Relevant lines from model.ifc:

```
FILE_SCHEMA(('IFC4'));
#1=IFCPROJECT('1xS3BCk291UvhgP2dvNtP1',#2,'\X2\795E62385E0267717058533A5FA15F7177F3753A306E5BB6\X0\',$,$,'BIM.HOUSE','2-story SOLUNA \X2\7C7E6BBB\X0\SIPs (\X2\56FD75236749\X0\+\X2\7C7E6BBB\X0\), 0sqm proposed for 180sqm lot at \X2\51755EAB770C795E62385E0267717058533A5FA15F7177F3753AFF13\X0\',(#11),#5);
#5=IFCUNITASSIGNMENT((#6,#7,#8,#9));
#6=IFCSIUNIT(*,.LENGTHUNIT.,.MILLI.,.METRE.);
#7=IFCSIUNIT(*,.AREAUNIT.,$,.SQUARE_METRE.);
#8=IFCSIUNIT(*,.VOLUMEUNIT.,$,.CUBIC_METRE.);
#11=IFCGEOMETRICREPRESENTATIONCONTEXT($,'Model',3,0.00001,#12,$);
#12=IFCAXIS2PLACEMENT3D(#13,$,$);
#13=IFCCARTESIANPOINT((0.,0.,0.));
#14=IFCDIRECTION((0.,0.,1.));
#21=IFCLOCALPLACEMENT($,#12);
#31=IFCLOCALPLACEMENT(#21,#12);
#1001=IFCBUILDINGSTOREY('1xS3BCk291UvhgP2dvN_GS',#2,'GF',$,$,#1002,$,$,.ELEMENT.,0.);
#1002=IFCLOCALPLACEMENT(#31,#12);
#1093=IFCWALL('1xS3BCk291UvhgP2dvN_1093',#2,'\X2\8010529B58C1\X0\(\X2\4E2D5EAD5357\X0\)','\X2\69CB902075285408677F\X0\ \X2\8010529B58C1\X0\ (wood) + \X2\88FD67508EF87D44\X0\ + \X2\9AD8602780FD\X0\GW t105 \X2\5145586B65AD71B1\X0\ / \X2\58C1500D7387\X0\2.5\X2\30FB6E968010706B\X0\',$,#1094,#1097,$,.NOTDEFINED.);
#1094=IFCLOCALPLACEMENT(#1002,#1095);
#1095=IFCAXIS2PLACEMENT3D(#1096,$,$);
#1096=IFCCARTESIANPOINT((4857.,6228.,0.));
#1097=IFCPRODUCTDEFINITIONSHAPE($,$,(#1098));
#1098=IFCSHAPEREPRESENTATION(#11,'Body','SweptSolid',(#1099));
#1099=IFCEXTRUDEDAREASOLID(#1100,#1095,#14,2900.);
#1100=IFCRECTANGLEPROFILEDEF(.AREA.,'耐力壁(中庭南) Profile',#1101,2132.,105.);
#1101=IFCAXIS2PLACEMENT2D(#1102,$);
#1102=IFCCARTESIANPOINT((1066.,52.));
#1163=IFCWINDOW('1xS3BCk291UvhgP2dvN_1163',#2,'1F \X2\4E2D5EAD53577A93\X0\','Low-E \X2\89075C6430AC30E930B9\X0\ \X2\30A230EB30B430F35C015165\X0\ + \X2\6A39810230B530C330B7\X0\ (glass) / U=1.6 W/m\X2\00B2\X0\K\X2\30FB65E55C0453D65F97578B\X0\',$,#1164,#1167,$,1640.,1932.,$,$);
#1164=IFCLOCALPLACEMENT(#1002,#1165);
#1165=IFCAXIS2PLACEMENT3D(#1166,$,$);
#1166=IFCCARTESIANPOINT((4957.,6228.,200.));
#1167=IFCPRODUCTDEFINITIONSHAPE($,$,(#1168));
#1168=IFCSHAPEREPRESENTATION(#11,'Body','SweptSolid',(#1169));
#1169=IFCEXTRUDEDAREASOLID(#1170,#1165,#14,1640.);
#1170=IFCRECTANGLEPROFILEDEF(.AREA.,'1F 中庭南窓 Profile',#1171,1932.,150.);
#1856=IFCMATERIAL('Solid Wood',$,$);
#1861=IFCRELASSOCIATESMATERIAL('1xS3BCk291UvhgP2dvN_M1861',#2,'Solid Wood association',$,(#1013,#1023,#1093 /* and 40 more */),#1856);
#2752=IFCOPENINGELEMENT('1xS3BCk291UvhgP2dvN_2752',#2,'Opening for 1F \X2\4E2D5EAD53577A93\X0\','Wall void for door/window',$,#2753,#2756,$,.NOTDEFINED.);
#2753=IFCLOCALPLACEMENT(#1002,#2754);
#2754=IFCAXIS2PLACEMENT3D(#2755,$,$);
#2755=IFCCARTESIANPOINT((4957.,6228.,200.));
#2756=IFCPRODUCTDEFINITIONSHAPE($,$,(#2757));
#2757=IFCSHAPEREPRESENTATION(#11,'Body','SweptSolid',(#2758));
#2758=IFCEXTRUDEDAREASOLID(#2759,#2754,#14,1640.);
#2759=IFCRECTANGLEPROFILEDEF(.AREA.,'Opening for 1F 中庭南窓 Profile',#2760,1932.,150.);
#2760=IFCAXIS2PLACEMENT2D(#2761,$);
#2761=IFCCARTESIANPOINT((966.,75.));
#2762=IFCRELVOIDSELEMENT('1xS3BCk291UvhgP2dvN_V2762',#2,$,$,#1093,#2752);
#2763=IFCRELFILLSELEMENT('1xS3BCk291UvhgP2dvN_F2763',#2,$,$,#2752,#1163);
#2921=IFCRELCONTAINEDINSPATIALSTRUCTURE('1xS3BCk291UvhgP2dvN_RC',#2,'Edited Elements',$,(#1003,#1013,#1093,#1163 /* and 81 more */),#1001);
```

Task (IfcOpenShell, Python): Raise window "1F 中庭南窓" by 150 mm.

```python
import numpy as np
import ifcopenshell
import ifcopenshell.api.geometry
import ifcopenshell.util.placement
import ifcopenshell.util.unit

model = ifcopenshell.open("model.ifc")
unit_scale = ifcopenshell.util.unit.calculate_unit_scale(model)

window = model.by_guid("1xS3BCk291UvhgP2dvN_1163")
opening = window.FillsVoids[0].RelatingOpeningElement
dz = 0.15 / unit_scale

shift = np.array([0.0, 0.0, dz])
# The window is not placed relative to its opening, so move both.
for product in (opening, window):
    matrix = ifcopenshell.util.placement.get_local_placement(product.ObjectPlacement)
    matrix[:3, 3] += shift
    ifcopenshell.api.geometry.edit_object_placement(model, product=product, matrix=matrix, is_si=False)

print(f"moved by {dz * unit_scale:+.3f} m")

model.write("model_updated.ifc")
```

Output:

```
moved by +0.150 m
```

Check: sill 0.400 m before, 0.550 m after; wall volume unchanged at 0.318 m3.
